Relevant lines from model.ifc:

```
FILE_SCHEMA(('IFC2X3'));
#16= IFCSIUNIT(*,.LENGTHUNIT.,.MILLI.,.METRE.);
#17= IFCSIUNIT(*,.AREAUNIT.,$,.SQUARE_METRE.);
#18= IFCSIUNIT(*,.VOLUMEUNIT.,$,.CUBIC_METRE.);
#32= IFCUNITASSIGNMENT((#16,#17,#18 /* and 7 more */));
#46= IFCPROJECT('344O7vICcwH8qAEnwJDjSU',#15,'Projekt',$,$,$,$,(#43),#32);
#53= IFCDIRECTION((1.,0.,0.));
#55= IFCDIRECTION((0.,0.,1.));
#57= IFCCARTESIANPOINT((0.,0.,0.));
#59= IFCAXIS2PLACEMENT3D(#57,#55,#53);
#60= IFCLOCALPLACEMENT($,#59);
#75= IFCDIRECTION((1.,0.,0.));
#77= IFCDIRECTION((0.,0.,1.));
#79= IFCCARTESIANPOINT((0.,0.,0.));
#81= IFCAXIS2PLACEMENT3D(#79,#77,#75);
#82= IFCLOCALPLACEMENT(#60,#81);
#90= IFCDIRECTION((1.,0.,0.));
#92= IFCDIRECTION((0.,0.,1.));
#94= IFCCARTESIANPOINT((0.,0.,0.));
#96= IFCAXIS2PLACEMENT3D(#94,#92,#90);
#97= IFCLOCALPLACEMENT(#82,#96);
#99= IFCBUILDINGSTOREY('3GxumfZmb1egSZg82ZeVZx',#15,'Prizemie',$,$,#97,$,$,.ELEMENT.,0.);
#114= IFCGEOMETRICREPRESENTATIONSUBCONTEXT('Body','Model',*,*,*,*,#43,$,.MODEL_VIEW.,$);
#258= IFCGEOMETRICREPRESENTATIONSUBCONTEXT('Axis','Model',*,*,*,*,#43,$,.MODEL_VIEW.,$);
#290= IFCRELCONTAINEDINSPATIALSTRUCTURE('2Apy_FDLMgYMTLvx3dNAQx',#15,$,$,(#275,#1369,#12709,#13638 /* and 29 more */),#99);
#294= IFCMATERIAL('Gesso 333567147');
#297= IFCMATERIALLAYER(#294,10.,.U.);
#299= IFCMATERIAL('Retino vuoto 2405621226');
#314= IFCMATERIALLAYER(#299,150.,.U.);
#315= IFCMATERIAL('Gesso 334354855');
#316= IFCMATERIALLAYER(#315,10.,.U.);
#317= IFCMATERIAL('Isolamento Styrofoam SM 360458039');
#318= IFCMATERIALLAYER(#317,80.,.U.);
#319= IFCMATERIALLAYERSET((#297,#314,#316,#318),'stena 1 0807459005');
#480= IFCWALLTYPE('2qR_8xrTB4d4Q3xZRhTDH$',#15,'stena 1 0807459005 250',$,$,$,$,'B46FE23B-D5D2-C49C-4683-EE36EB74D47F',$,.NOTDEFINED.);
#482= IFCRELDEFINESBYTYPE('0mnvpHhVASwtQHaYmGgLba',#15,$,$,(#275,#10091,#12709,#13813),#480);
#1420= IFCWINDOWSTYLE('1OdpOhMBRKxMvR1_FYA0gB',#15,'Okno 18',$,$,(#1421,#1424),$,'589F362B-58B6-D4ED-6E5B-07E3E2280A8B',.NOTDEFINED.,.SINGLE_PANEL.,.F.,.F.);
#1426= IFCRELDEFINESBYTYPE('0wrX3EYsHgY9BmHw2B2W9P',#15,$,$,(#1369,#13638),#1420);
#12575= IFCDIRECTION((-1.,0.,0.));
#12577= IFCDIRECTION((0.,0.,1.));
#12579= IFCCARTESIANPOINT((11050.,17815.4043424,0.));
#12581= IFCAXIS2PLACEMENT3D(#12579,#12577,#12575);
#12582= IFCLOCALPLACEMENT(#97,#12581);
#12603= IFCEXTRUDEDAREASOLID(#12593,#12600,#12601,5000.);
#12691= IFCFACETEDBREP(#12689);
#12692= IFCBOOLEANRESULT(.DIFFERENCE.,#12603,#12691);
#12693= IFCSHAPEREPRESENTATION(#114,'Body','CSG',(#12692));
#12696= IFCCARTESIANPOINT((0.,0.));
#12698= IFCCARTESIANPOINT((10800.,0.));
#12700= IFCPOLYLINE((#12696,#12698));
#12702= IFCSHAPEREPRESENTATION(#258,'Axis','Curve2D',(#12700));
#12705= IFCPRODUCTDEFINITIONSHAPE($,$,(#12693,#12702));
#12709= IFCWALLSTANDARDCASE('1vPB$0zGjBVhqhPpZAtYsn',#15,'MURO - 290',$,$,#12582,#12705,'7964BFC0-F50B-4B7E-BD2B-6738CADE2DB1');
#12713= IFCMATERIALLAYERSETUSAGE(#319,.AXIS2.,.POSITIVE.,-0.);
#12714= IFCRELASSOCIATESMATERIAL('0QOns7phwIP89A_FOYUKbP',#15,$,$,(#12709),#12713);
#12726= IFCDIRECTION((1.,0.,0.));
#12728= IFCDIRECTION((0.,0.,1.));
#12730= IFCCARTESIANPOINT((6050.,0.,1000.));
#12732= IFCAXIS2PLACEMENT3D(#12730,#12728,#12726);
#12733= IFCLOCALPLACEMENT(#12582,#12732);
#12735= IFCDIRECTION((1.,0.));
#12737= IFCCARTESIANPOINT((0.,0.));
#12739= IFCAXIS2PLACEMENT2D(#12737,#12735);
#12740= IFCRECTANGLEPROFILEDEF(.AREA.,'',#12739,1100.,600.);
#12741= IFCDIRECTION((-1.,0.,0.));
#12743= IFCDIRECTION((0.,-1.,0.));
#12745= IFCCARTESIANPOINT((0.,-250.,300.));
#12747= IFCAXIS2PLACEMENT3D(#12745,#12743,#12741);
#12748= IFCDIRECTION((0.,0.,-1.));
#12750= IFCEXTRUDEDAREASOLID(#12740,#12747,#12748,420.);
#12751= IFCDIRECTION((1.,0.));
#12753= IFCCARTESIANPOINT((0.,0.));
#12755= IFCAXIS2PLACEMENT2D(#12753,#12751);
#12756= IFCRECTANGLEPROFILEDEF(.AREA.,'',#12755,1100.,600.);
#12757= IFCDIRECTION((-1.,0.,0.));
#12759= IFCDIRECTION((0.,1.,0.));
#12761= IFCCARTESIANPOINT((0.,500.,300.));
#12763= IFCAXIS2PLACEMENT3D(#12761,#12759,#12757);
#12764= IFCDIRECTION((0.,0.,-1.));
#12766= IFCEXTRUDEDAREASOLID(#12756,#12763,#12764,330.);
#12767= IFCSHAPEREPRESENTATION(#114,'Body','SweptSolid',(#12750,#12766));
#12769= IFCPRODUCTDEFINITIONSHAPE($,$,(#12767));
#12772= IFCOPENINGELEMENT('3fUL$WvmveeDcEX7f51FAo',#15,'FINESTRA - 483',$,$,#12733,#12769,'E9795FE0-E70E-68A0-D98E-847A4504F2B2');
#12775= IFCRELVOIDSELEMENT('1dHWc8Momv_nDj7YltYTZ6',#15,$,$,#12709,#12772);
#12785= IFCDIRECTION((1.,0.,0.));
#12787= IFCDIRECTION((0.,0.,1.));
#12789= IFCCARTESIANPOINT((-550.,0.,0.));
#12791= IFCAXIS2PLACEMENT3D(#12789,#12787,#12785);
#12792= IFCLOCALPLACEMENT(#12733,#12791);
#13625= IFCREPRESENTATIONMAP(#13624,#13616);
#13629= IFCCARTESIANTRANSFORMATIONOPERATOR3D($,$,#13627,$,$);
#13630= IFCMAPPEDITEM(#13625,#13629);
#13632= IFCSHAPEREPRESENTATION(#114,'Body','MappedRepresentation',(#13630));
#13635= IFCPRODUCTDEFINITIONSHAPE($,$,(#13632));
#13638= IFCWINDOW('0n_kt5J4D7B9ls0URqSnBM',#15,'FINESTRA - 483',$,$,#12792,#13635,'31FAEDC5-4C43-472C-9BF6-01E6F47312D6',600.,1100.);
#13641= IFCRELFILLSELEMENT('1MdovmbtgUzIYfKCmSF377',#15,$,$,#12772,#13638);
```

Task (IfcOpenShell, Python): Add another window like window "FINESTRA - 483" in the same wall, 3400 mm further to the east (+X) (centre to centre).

```python
import ifcopenshell
import ifcopenshell.api.feature
import ifcopenshell.api.geometry
import ifcopenshell.api.root
import ifcopenshell.geom
import ifcopenshell.util.element
import ifcopenshell.util.placement
import ifcopenshell.util.shape

model = ifcopenshell.open("model.ifc")
settings = ifcopenshell.geom.settings()


def volume(element):
    """Net volume in cubic metres, openings subtracted."""
    shape = ifcopenshell.geom.create_shape(settings, element)
    return ifcopenshell.util.shape.get_volume(shape.geometry)


def reuse_history(source, copy):
    """copy_class also copies each property set's owner history, people and application; keep the originals."""
    for rel in copy.IsDefinedBy:
        if rel.is_a("IfcRelDefinesByProperties") and (history := rel.RelatingPropertyDefinition.OwnerHistory):
            rel.RelatingPropertyDefinition.OwnerHistory = source.OwnerHistory
            ifcopenshell.util.element.remove_deep2(model, history)


window = model.by_id(13638)
opening = window.FillsVoids[0].RelatingOpeningElement
wall = opening.VoidsElements[0].RelatingBuildingElement
before = volume(wall)
shift = ifcopenshell.util.placement.get_local_placement(wall.ObjectPlacement)[:3, 0] * -3400.0

# copy_class copies the void relationship, type, container and properties, but no geometry.
new_opening = ifcopenshell.api.root.copy_class(model, product=opening)
new_opening.Representation = ifcopenshell.util.element.copy_deep(
    model, opening.Representation, exclude=["IfcGeometricRepresentationContext", "IfcRepresentationMap"]
)
new_opening.Tag = None
new_window = ifcopenshell.api.root.copy_class(model, product=window)
new_window.Representation = ifcopenshell.util.element.copy_deep(
    model, window.Representation, exclude=["IfcGeometricRepresentationContext", "IfcRepresentationMap"]
)
new_window.Tag = None
reuse_history(window, new_window)
fills = ifcopenshell.api.feature.add_filling(model, opening=new_opening, element=new_window)
fills.OwnerHistory = new_window.OwnerHistory  # required in IFC2X3

for old, new in ((opening, new_opening), (window, new_window)):
    matrix = ifcopenshell.util.placement.get_local_placement(old.ObjectPlacement)
    matrix[:3, 3] += shift
    ifcopenshell.api.geometry.edit_object_placement(model, product=new, matrix=matrix, is_si=False)

after = volume(wall)

print(f"wall volume {before:.3f} -> {after:.3f} m3")

model.write("model-out.ifc")
```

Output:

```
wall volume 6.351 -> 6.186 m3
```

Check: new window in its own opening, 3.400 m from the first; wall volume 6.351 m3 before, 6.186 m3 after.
